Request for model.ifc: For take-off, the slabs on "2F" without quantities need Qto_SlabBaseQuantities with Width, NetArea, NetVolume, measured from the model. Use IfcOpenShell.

First a look at what the model holds.

```python
import ifcopenshell
import ifcopenshell.util.element
import ifcopenshell.util.unit

model = ifcopenshell.open("model.ifc")
print(model.schema)
for unit_type in ("LENGTHUNIT", "AREAUNIT", "VOLUMEUNIT"):
    print(unit_type, ifcopenshell.util.unit.calculate_unit_scale(model, unit_type))
storey = next(s for s in model.by_type("IfcBuildingStorey") if s.Name == "2F")
slabs = [e for e in ifcopenshell.util.element.get_decomposition(storey) if e.is_a("IfcSlab")]
for e in sorted(slabs, key=lambda e: e.id()):
    print(e.id(), e.is_a(), e.Name, list(ifcopenshell.util.element.get_psets(e, qtos_only=True)), sep=" | ")
```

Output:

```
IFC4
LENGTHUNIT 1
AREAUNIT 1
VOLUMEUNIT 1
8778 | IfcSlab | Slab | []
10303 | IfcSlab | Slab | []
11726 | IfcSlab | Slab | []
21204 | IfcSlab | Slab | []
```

```python
import ifcopenshell
import ifcopenshell.api.pset
import ifcopenshell.geom
import ifcopenshell.util.element
import ifcopenshell.util.shape
import ifcopenshell.util.unit

model = ifcopenshell.open("model.ifc")
unit_scale = ifcopenshell.util.unit.calculate_unit_scale(model)
area_scale = ifcopenshell.util.unit.calculate_unit_scale(model, "AREAUNIT")
volume_scale = ifcopenshell.util.unit.calculate_unit_scale(model, "VOLUMEUNIT")
settings = ifcopenshell.geom.settings()

storey = next(s for s in model.by_type("IfcBuildingStorey") if s.Name == "2F")
slabs = [e for e in ifcopenshell.util.element.get_decomposition(storey) if e.is_a("IfcSlab")]

for e in sorted(slabs, key=lambda e: e.id()):
    if ifcopenshell.util.element.get_psets(e, qtos_only=True, should_inherit=False):
        continue
    # Geometry comes back in metres, in the element's own axes.
    shape = ifcopenshell.geom.create_shape(settings, e)
    values = {
        "Width": ifcopenshell.util.shape.get_z(shape.geometry) / unit_scale,
        "NetArea": ifcopenshell.util.shape.get_footprint_area(shape.geometry) / area_scale,
        "NetVolume": ifcopenshell.util.shape.get_volume(shape.geometry) / volume_scale,
    }
    qto = ifcopenshell.api.pset.add_qto(model, product=e, name="Qto_SlabBaseQuantities")
    ifcopenshell.api.pset.edit_qto(model, qto=qto, properties=values)
    print(e.id(), {k: round(v, 3) for k, v in values.items()})

model.write("model_updated.ifc")
```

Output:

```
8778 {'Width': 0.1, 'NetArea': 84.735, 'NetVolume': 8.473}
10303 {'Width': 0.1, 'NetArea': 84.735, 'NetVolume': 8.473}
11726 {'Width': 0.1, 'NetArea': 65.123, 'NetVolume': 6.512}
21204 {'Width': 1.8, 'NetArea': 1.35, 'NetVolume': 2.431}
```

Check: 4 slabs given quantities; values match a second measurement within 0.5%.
